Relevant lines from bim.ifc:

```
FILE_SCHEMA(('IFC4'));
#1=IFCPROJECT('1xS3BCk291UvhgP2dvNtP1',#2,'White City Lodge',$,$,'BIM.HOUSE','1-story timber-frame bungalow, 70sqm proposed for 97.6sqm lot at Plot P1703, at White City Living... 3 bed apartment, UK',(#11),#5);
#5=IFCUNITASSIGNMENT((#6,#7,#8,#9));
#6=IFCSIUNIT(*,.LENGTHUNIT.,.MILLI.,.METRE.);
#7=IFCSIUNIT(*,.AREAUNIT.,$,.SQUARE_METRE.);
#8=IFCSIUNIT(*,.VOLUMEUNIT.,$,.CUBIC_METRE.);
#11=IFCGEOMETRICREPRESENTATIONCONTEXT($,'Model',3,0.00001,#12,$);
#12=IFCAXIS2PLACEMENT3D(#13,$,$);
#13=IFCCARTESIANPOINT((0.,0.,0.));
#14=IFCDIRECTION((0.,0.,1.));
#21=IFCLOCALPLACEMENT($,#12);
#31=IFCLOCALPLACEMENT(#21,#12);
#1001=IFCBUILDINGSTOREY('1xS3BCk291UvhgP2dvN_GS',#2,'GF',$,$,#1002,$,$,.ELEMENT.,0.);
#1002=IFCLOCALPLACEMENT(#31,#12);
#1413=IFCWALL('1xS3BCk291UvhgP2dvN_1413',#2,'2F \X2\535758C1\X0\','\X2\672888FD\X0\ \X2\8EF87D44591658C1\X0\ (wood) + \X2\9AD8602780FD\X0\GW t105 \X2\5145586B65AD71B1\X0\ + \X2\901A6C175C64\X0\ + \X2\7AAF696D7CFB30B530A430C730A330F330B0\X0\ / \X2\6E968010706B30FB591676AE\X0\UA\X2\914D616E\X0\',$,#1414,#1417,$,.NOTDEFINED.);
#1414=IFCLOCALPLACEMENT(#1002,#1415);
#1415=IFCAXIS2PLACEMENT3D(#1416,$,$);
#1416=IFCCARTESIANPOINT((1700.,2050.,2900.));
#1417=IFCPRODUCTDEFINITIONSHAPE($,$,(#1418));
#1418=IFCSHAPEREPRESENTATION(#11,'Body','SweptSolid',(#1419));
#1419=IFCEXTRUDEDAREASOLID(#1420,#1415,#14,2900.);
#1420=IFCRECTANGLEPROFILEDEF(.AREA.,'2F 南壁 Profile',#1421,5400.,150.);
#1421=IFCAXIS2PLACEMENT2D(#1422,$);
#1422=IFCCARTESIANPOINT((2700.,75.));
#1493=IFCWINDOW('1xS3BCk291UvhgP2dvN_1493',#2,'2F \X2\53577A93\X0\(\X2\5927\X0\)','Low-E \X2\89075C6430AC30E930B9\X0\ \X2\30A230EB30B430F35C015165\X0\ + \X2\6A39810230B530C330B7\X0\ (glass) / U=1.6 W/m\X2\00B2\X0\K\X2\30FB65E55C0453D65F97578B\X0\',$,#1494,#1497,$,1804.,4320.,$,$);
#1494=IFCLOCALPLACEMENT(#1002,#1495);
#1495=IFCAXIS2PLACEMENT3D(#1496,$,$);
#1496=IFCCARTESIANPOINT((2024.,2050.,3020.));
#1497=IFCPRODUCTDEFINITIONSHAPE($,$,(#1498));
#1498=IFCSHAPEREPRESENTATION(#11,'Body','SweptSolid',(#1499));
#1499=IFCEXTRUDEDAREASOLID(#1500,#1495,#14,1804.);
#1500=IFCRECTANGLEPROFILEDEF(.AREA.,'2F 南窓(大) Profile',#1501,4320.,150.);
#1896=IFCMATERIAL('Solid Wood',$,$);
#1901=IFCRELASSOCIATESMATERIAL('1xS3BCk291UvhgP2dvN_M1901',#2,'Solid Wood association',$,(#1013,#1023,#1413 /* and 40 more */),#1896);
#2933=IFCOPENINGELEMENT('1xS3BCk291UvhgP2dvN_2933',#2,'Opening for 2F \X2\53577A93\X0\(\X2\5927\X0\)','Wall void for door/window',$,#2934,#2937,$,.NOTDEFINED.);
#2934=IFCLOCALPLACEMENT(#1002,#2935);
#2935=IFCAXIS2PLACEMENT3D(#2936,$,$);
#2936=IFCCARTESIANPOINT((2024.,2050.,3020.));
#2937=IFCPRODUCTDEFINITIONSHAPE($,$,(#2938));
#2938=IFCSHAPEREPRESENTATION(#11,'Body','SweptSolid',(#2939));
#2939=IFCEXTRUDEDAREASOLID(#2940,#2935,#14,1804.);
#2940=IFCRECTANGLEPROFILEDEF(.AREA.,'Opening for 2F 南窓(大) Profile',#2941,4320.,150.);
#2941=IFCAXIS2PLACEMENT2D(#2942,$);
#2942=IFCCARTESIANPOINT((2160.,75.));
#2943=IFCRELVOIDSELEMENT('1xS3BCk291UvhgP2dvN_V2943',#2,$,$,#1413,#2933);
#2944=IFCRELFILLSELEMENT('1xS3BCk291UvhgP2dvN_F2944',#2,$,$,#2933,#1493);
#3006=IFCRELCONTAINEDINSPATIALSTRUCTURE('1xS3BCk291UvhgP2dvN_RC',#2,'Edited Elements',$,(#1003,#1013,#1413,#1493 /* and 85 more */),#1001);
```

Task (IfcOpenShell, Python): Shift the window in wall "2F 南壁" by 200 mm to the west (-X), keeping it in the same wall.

```python
import ifcopenshell
import ifcopenshell.api.geometry
import ifcopenshell.util.placement
import ifcopenshell.util.unit

model = ifcopenshell.open("bim.ifc")
unit_scale = ifcopenshell.util.unit.calculate_unit_scale(model)

window = model.by_guid("1xS3BCk291UvhgP2dvN_1493")
opening = window.FillsVoids[0].RelatingOpeningElement
wall = opening.VoidsElements[0].RelatingBuildingElement

wall_matrix = ifcopenshell.util.placement.get_local_placement(wall.ObjectPlacement)
shift = wall_matrix[:3, 0] * -0.2 / unit_scale
before = ifcopenshell.util.placement.get_local_placement(window.ObjectPlacement)[:3, 3].copy()

# The window is not placed relative to its opening, so move both.
for product in (opening, window):
    matrix = ifcopenshell.util.placement.get_local_placement(product.ObjectPlacement)
    matrix[:3, 3] += shift
    ifcopenshell.api.geometry.edit_object_placement(model, product=product, matrix=matrix, is_si=False)

after = ifcopenshell.util.placement.get_local_placement(window.ObjectPlacement)[:3, 3]
print("window moved by", (after - before).round(3) + 0.0)

model.write("bim_v2.ifc")
```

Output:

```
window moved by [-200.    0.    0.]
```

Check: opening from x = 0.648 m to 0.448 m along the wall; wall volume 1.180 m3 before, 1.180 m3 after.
